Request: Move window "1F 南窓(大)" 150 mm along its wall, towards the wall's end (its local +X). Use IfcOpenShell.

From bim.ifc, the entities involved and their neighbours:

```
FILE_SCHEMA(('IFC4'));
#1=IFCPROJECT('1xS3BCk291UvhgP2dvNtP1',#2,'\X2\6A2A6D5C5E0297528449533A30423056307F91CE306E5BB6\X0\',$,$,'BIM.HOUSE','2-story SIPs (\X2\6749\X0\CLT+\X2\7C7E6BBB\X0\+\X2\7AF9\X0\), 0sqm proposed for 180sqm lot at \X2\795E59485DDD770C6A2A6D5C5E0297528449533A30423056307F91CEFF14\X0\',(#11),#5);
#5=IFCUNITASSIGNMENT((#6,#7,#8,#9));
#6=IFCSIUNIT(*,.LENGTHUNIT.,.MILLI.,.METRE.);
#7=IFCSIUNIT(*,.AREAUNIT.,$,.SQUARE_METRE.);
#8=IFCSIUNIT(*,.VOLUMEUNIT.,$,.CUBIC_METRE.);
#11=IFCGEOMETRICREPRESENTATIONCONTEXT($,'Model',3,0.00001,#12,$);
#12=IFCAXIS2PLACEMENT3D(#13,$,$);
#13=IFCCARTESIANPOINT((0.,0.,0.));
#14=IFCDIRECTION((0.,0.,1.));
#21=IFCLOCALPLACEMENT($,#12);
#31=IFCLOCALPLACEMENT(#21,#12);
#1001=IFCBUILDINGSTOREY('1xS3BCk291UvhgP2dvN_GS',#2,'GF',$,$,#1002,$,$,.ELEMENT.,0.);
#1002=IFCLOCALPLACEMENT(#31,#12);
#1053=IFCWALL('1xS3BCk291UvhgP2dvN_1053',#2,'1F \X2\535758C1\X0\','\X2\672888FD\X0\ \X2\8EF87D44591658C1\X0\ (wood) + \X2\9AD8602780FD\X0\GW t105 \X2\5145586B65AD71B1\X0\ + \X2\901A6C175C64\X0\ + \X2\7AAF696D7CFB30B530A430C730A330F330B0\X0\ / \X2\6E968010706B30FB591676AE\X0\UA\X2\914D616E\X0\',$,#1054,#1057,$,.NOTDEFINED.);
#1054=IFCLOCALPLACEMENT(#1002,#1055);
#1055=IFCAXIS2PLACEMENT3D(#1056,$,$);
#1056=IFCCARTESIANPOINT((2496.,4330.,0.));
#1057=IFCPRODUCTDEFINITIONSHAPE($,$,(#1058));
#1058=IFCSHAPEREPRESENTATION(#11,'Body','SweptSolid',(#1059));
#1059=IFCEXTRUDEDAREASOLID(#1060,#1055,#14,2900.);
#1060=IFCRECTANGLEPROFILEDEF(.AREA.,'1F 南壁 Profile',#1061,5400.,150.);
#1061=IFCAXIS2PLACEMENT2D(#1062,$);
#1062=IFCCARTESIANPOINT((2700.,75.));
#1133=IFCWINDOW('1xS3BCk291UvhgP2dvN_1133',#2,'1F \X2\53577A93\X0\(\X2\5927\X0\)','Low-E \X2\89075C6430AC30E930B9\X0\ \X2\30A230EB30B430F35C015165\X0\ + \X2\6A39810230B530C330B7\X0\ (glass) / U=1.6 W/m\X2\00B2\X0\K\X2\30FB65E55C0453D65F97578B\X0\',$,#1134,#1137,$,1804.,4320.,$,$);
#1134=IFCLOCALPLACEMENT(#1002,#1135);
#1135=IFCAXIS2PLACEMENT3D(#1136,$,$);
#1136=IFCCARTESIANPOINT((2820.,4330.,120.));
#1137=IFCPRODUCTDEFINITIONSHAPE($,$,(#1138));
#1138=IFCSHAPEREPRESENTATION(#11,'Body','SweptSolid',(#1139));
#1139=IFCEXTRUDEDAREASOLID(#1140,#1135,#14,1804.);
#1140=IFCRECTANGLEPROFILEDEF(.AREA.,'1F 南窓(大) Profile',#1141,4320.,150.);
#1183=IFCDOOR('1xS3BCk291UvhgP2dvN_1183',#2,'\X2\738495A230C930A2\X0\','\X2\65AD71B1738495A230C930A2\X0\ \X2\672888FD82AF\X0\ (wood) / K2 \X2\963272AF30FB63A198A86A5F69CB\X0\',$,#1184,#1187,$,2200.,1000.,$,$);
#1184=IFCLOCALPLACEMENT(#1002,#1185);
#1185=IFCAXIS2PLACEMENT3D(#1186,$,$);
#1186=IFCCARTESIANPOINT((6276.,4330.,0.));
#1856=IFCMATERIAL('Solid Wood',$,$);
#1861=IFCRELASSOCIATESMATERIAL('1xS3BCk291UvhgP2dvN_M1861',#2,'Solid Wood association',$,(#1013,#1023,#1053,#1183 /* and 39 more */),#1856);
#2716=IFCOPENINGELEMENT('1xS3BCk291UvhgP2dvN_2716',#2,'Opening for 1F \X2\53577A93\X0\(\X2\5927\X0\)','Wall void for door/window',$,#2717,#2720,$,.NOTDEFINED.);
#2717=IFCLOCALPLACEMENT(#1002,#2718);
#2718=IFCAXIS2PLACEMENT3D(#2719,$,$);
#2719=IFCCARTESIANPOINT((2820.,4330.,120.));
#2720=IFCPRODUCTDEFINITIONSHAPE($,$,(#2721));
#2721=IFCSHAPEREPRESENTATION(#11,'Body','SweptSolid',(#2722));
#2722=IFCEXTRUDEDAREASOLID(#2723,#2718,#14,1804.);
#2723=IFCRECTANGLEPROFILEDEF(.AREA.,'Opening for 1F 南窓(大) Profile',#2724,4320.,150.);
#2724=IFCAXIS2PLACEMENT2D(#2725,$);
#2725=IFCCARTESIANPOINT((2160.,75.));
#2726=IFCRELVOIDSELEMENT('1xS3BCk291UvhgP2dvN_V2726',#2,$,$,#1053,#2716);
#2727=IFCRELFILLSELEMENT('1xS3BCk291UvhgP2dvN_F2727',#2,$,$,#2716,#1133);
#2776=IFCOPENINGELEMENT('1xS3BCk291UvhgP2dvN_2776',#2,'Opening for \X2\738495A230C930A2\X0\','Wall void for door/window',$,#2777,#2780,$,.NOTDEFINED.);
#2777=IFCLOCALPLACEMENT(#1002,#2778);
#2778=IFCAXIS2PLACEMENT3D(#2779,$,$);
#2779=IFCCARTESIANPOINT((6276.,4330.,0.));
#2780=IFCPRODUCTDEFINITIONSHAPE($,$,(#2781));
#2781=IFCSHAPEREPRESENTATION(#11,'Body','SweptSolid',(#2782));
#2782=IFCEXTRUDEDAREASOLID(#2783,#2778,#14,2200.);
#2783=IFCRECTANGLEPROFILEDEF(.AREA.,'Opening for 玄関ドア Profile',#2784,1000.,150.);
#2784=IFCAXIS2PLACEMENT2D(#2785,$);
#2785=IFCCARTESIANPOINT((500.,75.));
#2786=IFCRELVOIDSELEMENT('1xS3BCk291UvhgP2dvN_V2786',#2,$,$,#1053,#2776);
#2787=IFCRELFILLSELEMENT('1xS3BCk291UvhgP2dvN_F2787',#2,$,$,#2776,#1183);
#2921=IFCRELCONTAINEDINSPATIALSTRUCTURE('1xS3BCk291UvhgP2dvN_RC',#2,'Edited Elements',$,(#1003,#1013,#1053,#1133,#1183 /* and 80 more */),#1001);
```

```python
import ifcopenshell
import ifcopenshell.api.geometry
import ifcopenshell.util.placement

model = ifcopenshell.open("bim.ifc")

window = model.by_guid("1xS3BCk291UvhgP2dvN_1133")
opening = window.FillsVoids[0].RelatingOpeningElement
wall = opening.VoidsElements[0].RelatingBuildingElement

wall_matrix = ifcopenshell.util.placement.get_local_placement(wall.ObjectPlacement)
shift = wall_matrix[:3, 0] * 150.0
before = ifcopenshell.util.placement.get_local_placement(window.ObjectPlacement)[:3, 3].copy()

# The window is not placed relative to its opening, so move both.
for product in (opening, window):
    matrix = ifcopenshell.util.placement.get_local_placement(product.ObjectPlacement)
    matrix[:3, 3] += shift
    ifcopenshell.api.geometry.edit_object_placement(model, product=product, matrix=matrix, is_si=False)

after = ifcopenshell.util.placement.get_local_placement(window.ObjectPlacement)[:3, 3]
print("window moved by", (after - before).round(3) + 0.0)

model.write("bim_updated.ifc")
```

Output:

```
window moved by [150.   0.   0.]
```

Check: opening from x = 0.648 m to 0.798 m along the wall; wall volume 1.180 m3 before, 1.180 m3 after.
